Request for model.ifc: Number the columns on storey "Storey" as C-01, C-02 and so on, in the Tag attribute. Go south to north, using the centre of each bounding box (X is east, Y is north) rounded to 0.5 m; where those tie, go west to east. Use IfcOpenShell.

First a look at what the model holds.

```python
import ifcopenshell
import ifcopenshell.util.element
import ifcopenshell.util.placement

model = ifcopenshell.open("model.ifc")
print(model.schema)
storey = next(s for s in model.by_type("IfcBuildingStorey") if s.Name == "Storey")
columns = [e for e in ifcopenshell.util.element.get_decomposition(storey) if e.is_a("IfcColumn")]
for e in sorted(columns, key=lambda e: e.id()):
    origin = ifcopenshell.util.placement.get_local_placement(e.ObjectPlacement)[:3, 3]
    print(e.id(), e.Tag, e.Name, origin.round(2) + 0.0, sep=" | ")
```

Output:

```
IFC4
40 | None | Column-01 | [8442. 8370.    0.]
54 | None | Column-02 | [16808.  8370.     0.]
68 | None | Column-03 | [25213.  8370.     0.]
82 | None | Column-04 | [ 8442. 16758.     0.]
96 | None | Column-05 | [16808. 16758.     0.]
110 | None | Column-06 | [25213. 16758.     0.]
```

```python
import ifcopenshell
import ifcopenshell.geom
import ifcopenshell.util.element
import ifcopenshell.util.shape

model = ifcopenshell.open("model.ifc")
settings = ifcopenshell.geom.settings()
settings.set("use-world-coords", True)


def centre(element):
    shape = ifcopenshell.geom.create_shape(settings, element)
    return ifcopenshell.util.shape.get_bbox_centroid(shape.geometry)


storey = next(s for s in model.by_type("IfcBuildingStorey") if s.Name == "Storey")
columns = [e for e in ifcopenshell.util.element.get_decomposition(storey) if e.is_a("IfcColumn")]

# Insertion points can sit at a corner or the storey origin, so sort by the geometry (in metres).
centres = {e: centre(e) for e in columns}
columns.sort(key=lambda e: (round(centres[e][1] / 0.5), centres[e][0]))

for i, e in enumerate(columns, start=1):
    number = f"C-{i:02d}"
    e.Tag = number
    print(e.id(), number)

model.write("model_edited.ifc")
```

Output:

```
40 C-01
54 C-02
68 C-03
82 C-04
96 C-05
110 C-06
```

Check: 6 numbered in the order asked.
